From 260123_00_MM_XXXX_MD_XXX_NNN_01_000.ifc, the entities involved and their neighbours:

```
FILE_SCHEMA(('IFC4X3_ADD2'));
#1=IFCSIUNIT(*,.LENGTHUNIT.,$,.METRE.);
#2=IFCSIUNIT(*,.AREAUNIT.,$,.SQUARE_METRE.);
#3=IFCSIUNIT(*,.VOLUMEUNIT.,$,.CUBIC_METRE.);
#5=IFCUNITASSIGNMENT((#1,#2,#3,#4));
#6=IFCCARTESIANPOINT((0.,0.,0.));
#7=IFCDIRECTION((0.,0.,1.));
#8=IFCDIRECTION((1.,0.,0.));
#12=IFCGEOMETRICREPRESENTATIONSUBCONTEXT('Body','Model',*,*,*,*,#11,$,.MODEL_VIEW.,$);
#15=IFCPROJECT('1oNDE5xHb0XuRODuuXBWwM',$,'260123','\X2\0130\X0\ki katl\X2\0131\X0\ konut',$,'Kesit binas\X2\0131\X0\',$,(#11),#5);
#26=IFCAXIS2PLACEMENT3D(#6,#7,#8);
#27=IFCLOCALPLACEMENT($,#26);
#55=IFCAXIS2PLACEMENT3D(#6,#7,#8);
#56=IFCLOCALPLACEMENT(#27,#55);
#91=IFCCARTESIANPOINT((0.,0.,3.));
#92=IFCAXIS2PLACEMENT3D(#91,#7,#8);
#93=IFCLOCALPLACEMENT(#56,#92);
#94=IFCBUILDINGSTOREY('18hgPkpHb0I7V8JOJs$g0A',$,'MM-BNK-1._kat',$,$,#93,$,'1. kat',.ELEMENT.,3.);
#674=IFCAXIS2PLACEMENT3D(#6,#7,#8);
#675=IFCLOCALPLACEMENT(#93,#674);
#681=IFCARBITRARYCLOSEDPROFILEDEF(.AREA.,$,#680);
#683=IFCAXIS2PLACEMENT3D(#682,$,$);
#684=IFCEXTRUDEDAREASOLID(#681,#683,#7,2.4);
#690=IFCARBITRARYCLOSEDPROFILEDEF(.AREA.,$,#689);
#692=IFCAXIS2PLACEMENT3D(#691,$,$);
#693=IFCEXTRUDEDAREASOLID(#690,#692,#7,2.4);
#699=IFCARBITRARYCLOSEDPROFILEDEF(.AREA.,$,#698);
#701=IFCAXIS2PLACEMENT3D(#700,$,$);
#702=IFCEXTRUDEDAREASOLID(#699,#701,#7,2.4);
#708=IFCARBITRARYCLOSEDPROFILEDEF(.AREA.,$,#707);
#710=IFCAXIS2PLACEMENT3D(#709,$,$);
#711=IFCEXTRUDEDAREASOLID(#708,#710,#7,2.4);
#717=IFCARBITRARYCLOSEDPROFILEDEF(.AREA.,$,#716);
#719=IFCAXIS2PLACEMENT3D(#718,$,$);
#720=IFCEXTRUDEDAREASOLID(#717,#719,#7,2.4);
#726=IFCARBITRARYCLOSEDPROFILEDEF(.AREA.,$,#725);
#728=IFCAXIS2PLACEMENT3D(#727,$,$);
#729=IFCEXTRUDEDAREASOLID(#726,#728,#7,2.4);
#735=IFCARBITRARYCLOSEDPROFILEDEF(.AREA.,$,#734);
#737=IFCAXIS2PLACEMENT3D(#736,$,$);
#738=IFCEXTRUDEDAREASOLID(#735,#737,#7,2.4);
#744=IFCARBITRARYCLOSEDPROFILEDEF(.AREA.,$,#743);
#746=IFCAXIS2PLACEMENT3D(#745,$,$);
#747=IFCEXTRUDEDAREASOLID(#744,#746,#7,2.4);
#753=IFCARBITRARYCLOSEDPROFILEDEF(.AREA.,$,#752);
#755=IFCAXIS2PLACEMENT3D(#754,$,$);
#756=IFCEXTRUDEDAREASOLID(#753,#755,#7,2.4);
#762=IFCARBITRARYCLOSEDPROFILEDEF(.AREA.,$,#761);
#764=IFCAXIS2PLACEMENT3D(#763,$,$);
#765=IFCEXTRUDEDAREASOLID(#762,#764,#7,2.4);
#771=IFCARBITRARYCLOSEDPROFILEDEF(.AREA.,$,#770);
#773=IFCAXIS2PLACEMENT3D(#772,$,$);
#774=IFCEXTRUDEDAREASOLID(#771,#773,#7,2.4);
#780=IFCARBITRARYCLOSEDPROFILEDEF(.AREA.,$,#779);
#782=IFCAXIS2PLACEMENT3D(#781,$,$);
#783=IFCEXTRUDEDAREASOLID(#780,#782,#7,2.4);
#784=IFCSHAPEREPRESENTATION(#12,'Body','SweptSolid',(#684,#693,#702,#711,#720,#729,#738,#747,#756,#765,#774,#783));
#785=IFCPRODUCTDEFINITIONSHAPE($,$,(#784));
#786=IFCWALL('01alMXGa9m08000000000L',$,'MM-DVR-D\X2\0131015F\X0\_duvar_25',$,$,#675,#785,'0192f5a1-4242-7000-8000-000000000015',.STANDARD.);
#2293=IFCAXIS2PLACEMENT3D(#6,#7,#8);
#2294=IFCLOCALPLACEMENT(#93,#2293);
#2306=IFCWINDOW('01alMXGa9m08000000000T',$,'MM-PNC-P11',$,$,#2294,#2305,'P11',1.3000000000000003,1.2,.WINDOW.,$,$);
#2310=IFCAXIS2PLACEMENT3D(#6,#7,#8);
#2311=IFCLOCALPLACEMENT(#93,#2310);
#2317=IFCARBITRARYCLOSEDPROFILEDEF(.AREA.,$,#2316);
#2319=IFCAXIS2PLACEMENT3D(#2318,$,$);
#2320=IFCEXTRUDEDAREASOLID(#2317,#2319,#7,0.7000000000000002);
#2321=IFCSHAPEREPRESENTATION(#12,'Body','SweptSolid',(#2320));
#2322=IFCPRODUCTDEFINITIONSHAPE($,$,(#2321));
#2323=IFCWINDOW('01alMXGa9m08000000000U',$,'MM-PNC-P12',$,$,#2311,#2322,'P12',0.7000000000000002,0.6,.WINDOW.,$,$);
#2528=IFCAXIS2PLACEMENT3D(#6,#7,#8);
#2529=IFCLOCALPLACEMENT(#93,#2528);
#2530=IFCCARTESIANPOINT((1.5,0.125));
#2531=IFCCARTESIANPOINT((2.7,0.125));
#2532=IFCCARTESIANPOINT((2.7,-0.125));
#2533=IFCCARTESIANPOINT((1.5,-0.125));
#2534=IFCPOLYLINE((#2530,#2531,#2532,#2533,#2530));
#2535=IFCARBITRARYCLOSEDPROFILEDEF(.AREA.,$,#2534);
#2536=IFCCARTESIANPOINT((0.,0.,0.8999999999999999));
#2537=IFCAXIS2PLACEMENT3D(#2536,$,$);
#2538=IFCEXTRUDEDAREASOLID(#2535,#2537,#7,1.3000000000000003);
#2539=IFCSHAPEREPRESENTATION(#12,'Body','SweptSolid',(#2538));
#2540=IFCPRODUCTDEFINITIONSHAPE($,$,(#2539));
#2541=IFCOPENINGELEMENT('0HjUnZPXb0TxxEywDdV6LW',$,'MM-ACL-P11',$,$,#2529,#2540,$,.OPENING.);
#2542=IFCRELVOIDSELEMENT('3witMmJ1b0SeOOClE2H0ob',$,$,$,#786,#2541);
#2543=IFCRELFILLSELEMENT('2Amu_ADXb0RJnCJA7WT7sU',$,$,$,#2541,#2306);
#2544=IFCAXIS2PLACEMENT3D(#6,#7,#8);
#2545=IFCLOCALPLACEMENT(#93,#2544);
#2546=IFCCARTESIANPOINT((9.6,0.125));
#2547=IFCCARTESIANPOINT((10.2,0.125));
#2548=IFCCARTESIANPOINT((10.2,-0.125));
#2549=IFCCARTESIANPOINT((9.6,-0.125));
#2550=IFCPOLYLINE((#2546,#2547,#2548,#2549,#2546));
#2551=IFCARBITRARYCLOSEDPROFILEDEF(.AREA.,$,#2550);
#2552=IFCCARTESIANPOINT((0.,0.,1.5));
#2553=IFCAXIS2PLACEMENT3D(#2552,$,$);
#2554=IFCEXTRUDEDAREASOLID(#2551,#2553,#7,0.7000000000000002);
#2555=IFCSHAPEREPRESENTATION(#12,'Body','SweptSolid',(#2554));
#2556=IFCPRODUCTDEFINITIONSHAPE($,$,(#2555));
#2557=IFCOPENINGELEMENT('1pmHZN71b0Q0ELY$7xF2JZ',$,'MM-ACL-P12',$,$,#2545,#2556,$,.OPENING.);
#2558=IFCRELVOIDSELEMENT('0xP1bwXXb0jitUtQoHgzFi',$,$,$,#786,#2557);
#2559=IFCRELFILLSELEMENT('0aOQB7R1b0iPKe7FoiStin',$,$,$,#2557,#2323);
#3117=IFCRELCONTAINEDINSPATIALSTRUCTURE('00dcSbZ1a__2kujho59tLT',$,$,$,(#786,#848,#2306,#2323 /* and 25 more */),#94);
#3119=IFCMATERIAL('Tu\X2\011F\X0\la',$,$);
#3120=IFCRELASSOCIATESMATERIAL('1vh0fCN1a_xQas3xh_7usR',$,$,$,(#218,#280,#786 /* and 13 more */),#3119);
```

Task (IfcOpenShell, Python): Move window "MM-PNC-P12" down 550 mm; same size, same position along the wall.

```python
import numpy as np
import ifcopenshell
import ifcopenshell.api.geometry
import ifcopenshell.util.placement
import ifcopenshell.util.unit

model = ifcopenshell.open("260123_00_MM_XXXX_MD_XXX_NNN_01_000.ifc")
unit_scale = ifcopenshell.util.unit.calculate_unit_scale(model)

window = model.by_guid("01alMXGa9m08000000000U")
opening = window.FillsVoids[0].RelatingOpeningElement
dz = -0.55

shift = np.array([0.0, 0.0, dz])
# The window is not placed relative to its opening, so move both.
for product in (opening, window):
    matrix = ifcopenshell.util.placement.get_local_placement(product.ObjectPlacement)
    matrix[:3, 3] += shift
    ifcopenshell.api.geometry.edit_object_placement(model, product=product, matrix=matrix, is_si=False)

print(f"moved by {dz * unit_scale:+.3f} m")

model.write("260123_00_MM_XXXX_MD_XXX_NNN_01_000_updated.ifc")
```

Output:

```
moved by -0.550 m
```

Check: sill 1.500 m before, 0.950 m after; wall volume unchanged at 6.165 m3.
